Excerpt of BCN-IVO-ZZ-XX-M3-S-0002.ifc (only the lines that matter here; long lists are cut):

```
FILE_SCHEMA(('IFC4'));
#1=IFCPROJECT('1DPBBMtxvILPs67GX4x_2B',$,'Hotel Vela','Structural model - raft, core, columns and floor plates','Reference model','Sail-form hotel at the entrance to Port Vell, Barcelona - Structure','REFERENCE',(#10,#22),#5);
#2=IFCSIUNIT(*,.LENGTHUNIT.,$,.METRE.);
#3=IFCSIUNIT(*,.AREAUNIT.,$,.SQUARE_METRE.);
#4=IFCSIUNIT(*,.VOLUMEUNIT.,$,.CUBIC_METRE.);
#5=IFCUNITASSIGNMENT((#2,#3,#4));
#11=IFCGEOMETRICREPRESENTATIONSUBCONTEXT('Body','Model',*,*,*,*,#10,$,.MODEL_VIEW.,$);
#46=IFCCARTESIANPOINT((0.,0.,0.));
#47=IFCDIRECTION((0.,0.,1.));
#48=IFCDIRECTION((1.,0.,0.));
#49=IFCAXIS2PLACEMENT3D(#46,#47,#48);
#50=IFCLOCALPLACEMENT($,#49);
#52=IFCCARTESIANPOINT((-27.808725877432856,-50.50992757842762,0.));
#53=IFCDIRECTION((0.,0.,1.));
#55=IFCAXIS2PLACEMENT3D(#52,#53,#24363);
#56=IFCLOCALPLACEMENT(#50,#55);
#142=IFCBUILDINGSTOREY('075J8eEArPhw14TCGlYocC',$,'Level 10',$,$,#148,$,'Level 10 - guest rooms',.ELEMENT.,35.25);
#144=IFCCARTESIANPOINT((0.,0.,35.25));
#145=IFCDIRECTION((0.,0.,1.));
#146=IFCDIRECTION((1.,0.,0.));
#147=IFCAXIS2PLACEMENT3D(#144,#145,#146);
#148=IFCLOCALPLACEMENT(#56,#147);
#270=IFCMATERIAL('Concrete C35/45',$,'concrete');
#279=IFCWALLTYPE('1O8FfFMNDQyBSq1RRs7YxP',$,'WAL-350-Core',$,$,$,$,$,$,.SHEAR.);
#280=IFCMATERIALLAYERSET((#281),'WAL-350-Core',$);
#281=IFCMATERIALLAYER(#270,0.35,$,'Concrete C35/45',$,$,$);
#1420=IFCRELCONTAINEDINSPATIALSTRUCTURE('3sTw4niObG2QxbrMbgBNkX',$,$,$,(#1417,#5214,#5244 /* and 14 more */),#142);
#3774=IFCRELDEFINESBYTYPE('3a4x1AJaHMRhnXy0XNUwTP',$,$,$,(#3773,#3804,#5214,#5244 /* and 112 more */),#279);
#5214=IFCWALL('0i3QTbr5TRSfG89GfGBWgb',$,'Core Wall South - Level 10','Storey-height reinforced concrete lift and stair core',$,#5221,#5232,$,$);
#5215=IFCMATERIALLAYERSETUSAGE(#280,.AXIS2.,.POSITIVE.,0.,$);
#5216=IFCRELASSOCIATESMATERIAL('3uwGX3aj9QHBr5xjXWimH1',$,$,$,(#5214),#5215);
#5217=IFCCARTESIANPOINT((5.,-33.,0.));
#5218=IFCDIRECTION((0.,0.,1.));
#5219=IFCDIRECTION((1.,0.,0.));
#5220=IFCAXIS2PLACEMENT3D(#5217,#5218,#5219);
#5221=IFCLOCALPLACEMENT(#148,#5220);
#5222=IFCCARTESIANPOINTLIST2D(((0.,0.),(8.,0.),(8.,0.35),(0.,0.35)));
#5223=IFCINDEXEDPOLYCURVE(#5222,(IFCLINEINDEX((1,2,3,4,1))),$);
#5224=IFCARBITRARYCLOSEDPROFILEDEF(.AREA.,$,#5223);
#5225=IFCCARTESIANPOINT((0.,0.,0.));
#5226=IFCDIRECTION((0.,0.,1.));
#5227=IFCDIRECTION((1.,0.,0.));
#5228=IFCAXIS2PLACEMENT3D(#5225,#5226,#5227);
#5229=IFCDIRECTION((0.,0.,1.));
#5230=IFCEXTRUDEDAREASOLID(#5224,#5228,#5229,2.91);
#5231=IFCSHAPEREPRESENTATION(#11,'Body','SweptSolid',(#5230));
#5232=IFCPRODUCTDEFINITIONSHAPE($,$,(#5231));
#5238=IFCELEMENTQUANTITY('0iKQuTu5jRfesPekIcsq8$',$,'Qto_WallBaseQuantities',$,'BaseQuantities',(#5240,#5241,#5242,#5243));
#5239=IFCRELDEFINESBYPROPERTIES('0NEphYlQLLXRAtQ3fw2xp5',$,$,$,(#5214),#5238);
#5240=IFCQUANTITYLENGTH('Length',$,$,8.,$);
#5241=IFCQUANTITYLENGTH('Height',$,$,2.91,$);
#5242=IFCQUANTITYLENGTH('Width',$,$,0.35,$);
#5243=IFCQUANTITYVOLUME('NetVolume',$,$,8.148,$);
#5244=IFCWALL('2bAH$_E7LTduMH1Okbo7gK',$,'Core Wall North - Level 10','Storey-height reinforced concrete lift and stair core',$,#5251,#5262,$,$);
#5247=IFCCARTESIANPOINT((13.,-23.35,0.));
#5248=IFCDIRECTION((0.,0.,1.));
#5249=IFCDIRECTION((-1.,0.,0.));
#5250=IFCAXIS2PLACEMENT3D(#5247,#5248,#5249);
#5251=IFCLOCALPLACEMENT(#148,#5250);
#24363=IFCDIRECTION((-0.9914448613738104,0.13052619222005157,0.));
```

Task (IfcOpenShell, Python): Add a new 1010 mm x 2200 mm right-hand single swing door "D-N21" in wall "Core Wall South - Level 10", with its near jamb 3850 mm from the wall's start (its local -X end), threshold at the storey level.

```python
import numpy as np
import ifcopenshell
import ifcopenshell.api.feature
import ifcopenshell.api.geometry
import ifcopenshell.api.pset
import ifcopenshell.api.root
import ifcopenshell.api.spatial
import ifcopenshell.geom
import ifcopenshell.util.element
import ifcopenshell.util.placement
import ifcopenshell.util.representation
import ifcopenshell.util.shape
import ifcopenshell.util.unit

model = ifcopenshell.open("BCN-IVO-ZZ-XX-M3-S-0002.ifc")
unit_scale = ifcopenshell.util.unit.calculate_unit_scale(model)
volume_scale = ifcopenshell.util.unit.calculate_unit_scale(model, "VOLUMEUNIT")
settings = ifcopenshell.geom.settings()


def volume(element):
    """Net volume in cubic metres, openings subtracted."""
    shape = ifcopenshell.geom.create_shape(settings, element)
    return ifcopenshell.util.shape.get_volume(shape.geometry)


wall = model.by_id(5214)
storey = ifcopenshell.util.element.get_container(wall, ifc_class="IfcBuildingStorey")
context = ifcopenshell.util.representation.get_context(model, "Model", "Body", "MODEL_VIEW")
before = volume(wall)

width, height, from_end, sill = 1.01, 2.2, 3.85, 0.0  # metres

# The wall runs along its own X axis, and the end named is its -X end.
wall_shape = ifcopenshell.geom.create_shape(settings, wall)
x, y, z = ifcopenshell.util.shape.get_vertices(wall_shape.geometry).T
start = x.min() + from_end
face, thickness = float(y.min()), float(y.max() - y.min())
wall_matrix = ifcopenshell.util.placement.get_local_placement(wall.ObjectPlacement)
level = ifcopenshell.util.placement.get_local_placement(storey.ObjectPlacement)[2, 3]


def in_wall(x, y):
    """Placement at x, y metres in the wall's axes, at sill height."""
    matrix = wall_matrix.copy()
    matrix[:, 3] = wall_matrix @ np.array([x / unit_scale, y / unit_scale, 0.0, 1.0])
    matrix[2, 3] = level + sill / unit_scale
    return matrix


# Opening: a box that overshoots both wall faces by 50 mm.
opening = ifcopenshell.api.root.create_entity(model, ifc_class="IfcOpeningElement", predefined_type="OPENING")
box = ifcopenshell.api.geometry.add_wall_representation(
    model, context=context, length=width, height=height, thickness=thickness + 0.1
)
ifcopenshell.api.geometry.assign_representation(model, product=opening, representation=box)
ifcopenshell.api.geometry.edit_object_placement(model, product=opening, matrix=in_wall(start, face - 0.05), is_si=False)
ifcopenshell.api.feature.add_feature(model, feature=opening, element=wall)

door = ifcopenshell.api.root.create_entity(model, ifc_class="IfcDoor", name="D-N21", predefined_type="DOOR")
door.OverallWidth, door.OverallHeight = width / unit_scale, height / unit_scale
door.OperationType = "SINGLE_SWING_RIGHT"
body = ifcopenshell.api.geometry.add_door_representation(
    model,
    context=context,
    overall_width=door.OverallWidth,
    overall_height=door.OverallHeight,
    operation_type="SINGLE_SWING_RIGHT",
    lining_properties={"LiningDepth": thickness / unit_scale, "ThresholdDepth": thickness / unit_scale},
)
ifcopenshell.api.geometry.assign_representation(model, product=door, representation=body)
ifcopenshell.api.spatial.assign_container(model, products=[door], relating_structure=storey)
ifcopenshell.api.feature.add_filling(model, opening=opening, element=door)

# The lining spans the wall, so the door starts at the wall face.
ifcopenshell.api.geometry.edit_object_placement(model, product=door, matrix=in_wall(start, face), is_si=False)

after = volume(wall)

# Update the wall's stored quantities.
qto = model.by_id(ifcopenshell.util.element.get_pset(wall, "Qto_WallBaseQuantities", should_inherit=False)["id"])
ifcopenshell.api.pset.edit_qto(model, qto=qto, properties={"NetVolume": after / volume_scale})

print(f"wall volume {before:.3f} -> {after:.3f} m3")

model.write("BCN-IVO-ZZ-XX-M3-S-0002-out.ifc")
```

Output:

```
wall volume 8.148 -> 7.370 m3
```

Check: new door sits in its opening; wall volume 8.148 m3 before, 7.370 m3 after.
